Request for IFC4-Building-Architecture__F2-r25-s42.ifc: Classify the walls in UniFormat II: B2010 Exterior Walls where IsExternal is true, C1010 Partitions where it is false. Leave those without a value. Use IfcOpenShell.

First a look at what the model holds.

```python
import ifcopenshell
import ifcopenshell.util.element

model = ifcopenshell.open("IFC4-Building-Architecture__F2-r25-s42.ifc")
print(model.schema)
print("classifications:", [c.Name for c in model.by_type("IfcClassification")])
values = [ifcopenshell.util.element.get_pset(e, "Pset_WallCommon", "IsExternal") for e in model.by_type("IfcWall")]
for value in (True, False, None):
    print("IsExternal", value, values.count(value))
```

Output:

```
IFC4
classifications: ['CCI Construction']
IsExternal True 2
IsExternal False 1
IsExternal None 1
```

```python
import ifcopenshell
import ifcopenshell.api.classification
import ifcopenshell.util.element

model = ifcopenshell.open("IFC4-Building-Architecture__F2-r25-s42.ifc")

system = ifcopenshell.api.classification.add_classification(model, classification="UniFormat II")

walls = model.by_type("IfcWall")
external = {e: ifcopenshell.util.element.get_pset(e, "Pset_WallCommon", "IsExternal") for e in walls}
for flag, code, name in ((True, "B2010", "Exterior Walls"), (False, "C1010", "Partitions")):
    products = [e for e in walls if external[e] is flag]
    ifcopenshell.api.classification.add_reference(
        model, products=products, classification=system, identification=code, name=name
    )
    print(code, len(products))

model.write("IFC4-Building-Architecture__F2-r25-s42_v2.ifc")
```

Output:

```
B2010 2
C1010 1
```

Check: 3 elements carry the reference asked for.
